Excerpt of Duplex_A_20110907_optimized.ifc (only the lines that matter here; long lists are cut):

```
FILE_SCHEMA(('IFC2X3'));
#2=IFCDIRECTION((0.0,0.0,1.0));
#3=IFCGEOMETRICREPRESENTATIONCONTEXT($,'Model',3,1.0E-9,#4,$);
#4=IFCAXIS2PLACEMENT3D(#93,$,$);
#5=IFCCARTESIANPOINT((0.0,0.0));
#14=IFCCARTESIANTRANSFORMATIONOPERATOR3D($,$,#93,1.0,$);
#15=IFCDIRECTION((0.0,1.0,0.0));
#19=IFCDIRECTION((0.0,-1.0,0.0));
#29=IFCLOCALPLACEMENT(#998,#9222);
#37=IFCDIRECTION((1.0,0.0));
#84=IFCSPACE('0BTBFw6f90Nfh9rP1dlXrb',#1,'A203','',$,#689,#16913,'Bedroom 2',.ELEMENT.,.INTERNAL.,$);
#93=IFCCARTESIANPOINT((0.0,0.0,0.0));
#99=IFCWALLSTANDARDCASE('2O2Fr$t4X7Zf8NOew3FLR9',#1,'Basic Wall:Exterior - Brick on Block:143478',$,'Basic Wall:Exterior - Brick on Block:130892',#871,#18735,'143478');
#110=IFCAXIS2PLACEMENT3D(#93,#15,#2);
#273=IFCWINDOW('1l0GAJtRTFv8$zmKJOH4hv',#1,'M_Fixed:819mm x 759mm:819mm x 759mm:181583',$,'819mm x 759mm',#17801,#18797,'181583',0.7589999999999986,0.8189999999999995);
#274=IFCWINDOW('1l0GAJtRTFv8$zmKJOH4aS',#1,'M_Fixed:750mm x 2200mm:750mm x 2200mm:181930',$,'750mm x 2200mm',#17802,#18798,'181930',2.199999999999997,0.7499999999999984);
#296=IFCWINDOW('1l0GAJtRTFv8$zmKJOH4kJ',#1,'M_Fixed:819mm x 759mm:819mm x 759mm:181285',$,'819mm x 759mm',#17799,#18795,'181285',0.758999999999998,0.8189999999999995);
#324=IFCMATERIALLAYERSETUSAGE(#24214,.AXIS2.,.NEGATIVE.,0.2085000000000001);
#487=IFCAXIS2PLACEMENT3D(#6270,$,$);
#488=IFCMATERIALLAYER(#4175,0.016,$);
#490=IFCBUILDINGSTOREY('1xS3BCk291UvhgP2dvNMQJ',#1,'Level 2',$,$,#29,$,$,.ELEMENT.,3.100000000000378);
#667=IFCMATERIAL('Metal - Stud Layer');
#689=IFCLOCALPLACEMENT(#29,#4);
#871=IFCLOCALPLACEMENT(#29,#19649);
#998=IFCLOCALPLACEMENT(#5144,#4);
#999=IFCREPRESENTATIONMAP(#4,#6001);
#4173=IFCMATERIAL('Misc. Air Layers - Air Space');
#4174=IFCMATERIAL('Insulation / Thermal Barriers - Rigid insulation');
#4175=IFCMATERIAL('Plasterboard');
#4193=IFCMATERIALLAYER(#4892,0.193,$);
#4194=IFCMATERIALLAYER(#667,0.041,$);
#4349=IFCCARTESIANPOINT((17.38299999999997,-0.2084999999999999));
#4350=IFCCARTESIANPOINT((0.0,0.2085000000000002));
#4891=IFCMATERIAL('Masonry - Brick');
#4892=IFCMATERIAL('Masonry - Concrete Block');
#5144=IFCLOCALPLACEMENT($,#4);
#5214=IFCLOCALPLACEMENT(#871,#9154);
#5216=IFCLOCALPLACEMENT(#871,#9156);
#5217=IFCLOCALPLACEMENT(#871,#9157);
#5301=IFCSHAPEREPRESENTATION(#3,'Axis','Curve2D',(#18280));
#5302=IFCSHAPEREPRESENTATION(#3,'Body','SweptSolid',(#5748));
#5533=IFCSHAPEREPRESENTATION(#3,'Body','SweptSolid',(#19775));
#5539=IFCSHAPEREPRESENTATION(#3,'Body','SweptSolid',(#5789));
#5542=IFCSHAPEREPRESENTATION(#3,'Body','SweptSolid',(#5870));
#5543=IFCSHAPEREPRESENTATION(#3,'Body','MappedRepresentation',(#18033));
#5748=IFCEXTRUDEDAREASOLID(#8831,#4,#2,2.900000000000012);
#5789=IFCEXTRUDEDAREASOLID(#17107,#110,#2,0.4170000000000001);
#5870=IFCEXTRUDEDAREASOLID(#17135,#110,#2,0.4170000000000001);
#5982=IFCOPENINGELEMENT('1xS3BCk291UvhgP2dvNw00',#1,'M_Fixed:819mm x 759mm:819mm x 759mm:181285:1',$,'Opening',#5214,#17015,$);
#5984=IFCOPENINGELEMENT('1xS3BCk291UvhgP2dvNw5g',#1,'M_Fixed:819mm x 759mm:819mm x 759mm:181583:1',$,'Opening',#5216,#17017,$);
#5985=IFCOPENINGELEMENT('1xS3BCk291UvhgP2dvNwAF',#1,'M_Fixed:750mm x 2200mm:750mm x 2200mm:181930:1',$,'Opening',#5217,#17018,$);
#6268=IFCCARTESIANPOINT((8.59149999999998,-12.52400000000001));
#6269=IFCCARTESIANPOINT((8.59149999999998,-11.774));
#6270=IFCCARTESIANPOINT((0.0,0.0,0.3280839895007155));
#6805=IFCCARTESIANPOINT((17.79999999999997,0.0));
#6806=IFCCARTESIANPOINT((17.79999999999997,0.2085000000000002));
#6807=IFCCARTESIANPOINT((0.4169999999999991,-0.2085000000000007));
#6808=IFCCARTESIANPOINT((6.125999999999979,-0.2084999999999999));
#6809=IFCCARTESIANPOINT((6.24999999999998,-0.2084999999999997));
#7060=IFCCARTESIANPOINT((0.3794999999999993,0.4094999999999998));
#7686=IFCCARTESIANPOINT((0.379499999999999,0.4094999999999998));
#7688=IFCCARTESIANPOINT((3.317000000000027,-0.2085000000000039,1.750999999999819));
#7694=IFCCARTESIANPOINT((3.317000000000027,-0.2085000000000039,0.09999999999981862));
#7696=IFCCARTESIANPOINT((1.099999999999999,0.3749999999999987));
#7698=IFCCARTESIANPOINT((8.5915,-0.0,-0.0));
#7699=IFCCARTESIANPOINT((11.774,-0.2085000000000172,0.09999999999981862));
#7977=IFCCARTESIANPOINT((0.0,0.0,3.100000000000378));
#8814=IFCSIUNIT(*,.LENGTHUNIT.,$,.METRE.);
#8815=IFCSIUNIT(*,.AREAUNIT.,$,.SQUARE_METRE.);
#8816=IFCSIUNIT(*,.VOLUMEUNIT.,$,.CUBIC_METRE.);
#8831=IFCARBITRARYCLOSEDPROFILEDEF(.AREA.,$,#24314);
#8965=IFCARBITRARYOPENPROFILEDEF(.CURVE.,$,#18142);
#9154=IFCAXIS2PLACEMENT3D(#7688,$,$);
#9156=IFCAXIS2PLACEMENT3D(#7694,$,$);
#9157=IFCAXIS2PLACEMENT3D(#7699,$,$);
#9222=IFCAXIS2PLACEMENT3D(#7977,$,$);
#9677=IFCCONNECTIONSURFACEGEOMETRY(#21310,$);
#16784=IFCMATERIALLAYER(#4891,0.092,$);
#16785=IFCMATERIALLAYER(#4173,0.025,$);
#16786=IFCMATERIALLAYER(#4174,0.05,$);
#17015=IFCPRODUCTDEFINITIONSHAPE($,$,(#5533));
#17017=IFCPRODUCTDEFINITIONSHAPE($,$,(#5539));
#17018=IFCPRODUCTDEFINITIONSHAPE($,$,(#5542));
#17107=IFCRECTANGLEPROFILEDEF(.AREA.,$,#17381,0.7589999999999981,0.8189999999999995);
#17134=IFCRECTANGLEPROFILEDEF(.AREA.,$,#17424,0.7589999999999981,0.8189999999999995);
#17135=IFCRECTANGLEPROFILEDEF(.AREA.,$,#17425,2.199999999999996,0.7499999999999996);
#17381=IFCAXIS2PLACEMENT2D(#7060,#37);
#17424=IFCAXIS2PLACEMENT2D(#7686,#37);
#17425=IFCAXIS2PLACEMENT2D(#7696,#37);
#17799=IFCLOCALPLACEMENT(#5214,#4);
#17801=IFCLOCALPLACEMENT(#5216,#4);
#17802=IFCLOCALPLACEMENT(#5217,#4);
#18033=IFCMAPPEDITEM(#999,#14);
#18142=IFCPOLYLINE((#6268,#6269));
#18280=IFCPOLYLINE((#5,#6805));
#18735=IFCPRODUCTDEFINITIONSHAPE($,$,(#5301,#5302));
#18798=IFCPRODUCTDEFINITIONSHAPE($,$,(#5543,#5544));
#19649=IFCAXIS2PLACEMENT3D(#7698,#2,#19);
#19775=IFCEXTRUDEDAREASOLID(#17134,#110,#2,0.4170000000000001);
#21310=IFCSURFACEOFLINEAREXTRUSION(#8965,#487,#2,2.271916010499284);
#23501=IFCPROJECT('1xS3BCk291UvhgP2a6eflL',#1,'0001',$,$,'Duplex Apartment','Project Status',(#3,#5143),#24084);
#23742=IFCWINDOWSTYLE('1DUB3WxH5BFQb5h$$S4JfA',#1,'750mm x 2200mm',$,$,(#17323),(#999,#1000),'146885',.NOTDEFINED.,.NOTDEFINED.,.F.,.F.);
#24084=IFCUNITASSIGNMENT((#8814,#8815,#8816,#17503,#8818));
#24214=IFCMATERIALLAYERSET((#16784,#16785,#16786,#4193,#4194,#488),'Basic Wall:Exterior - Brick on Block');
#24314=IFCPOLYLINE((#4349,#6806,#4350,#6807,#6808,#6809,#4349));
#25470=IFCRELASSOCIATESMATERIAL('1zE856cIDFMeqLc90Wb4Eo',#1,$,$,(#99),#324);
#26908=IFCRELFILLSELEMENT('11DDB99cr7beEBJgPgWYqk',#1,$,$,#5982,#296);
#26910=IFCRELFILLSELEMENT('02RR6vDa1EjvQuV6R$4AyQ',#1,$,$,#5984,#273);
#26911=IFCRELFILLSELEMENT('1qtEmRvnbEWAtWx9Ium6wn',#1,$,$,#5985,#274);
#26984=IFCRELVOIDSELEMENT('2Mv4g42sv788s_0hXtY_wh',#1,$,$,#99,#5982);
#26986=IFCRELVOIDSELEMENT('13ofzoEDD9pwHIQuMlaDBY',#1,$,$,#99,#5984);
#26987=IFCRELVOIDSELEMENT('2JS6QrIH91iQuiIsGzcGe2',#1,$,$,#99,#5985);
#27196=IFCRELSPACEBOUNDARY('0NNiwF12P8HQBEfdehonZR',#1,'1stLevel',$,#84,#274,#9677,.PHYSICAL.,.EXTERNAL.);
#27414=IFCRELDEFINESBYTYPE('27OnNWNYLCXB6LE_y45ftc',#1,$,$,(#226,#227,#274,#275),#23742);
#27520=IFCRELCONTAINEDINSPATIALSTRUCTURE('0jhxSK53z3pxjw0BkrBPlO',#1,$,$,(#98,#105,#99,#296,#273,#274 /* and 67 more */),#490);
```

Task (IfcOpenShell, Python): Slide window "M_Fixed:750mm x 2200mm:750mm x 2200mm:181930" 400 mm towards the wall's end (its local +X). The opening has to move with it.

```python
import numpy as np
import ifcopenshell
import ifcopenshell.api.geometry
import ifcopenshell.util.placement
import ifcopenshell.util.unit

model = ifcopenshell.open("Duplex_A_20110907_optimized.ifc")
unit_scale = ifcopenshell.util.unit.calculate_unit_scale(model)

window = model.by_guid("1l0GAJtRTFv8$zmKJOH4aS")
opening = window.FillsVoids[0].RelatingOpeningElement
wall = opening.VoidsElements[0].RelatingBuildingElement

wall_matrix = ifcopenshell.util.placement.get_local_placement(wall.ObjectPlacement)
shift = wall_matrix[:3, 0] * 0.4 / unit_scale
before = ifcopenshell.util.placement.get_local_placement(window.ObjectPlacement)[:3, 3].copy()

# The window is placed relative to its opening, so it follows when the opening moves.
matrix = ifcopenshell.util.placement.get_local_placement(opening.ObjectPlacement)
matrix[:3, 3] += shift
ifcopenshell.api.geometry.edit_object_placement(
    model, product=opening, matrix=matrix, is_si=False, should_transform_children=True
)

# Space boundary surfaces are stored in each space's coordinates; move them too.
for rel in window.ProvidesBoundaries:
    if not rel.ConnectionGeometry:
        continue
    surface = rel.ConnectionGeometry.SurfaceOnRelatingElement
    space_matrix = ifcopenshell.util.placement.get_local_placement(rel.RelatingSpace.ObjectPlacement)
    point = np.array(surface.Position.Location.Coordinates) + space_matrix[:3, :3].T @ shift
    surface.Position = model.createIfcAxis2Placement3D(
        model.createIfcCartesianPoint(point.tolist()), surface.Position.Axis, surface.Position.RefDirection
    )

after = ifcopenshell.util.placement.get_local_placement(window.ObjectPlacement)[:3, 3]
print("window moved by", (after - before).round(3) + 0.0)

model.write("Duplex_A_20110907_optimized_v2.ifc")
```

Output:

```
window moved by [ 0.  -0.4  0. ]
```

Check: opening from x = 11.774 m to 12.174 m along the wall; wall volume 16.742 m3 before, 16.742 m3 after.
